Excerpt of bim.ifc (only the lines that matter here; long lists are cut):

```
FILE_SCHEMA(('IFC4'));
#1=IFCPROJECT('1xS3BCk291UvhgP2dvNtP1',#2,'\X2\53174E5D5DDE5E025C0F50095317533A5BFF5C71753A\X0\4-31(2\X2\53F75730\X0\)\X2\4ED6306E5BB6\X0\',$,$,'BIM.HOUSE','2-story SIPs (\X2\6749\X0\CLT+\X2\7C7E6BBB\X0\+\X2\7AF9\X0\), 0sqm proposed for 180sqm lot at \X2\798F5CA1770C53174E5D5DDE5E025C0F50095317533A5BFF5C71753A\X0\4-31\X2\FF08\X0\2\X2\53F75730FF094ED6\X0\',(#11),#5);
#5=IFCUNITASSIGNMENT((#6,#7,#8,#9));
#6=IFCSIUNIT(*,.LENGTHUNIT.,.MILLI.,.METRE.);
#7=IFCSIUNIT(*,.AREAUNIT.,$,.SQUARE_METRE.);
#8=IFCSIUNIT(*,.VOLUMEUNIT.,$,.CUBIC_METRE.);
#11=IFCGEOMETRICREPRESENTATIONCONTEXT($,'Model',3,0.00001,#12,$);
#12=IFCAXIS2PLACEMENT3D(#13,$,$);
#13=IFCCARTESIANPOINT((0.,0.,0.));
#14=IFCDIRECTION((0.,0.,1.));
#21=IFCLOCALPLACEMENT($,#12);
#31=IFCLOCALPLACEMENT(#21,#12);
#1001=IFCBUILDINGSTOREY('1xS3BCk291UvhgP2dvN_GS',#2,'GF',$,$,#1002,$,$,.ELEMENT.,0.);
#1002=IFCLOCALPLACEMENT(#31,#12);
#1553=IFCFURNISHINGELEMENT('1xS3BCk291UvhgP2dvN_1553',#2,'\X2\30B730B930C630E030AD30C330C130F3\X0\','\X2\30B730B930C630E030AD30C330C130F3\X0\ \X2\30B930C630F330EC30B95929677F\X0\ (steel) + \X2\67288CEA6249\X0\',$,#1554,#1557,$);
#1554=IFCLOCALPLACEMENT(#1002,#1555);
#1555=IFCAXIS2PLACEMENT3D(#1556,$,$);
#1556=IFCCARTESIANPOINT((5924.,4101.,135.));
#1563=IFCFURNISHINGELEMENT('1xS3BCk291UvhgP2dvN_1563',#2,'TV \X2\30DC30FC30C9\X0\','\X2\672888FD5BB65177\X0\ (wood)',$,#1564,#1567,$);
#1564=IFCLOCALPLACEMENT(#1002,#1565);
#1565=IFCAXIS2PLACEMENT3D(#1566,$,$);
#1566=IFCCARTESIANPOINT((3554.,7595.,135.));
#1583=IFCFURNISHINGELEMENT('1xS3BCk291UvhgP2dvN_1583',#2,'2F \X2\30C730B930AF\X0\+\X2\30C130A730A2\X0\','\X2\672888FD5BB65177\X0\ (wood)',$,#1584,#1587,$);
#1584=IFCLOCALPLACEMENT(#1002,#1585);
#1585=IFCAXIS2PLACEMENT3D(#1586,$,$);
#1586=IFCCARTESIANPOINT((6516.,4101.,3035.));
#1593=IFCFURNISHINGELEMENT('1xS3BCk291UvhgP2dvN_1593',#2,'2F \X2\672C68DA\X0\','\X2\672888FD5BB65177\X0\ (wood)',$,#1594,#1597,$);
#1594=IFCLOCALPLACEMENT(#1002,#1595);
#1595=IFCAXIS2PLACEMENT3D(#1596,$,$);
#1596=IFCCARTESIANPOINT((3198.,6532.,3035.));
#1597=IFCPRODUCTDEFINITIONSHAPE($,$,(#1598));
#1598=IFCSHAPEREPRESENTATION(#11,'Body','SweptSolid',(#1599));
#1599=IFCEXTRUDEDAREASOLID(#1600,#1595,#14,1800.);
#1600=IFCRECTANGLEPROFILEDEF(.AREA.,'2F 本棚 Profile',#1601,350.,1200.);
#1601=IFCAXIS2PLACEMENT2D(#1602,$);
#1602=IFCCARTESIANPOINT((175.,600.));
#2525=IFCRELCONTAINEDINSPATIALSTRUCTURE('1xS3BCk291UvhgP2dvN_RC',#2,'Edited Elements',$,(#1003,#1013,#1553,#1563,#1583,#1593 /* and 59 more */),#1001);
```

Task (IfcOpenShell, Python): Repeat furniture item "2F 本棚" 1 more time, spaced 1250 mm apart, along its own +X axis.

```python
import ifcopenshell
import ifcopenshell.api.geometry
import ifcopenshell.api.root
import ifcopenshell.util.element
import ifcopenshell.util.placement
import ifcopenshell.util.unit

model = ifcopenshell.open("bim.ifc")
unit_scale = ifcopenshell.util.unit.calculate_unit_scale(model)


def reuse_history(source, copy):
    """copy_class also copies each property set's owner history, people and application; keep the originals."""
    for rel in copy.IsDefinedBy:
        if rel.is_a("IfcRelDefinesByProperties") and (history := rel.RelatingPropertyDefinition.OwnerHistory):
            rel.RelatingPropertyDefinition.OwnerHistory = source.OwnerHistory
            ifcopenshell.util.element.remove_deep2(model, history)


source = model.by_guid("1xS3BCk291UvhgP2dvN_1593")
base = ifcopenshell.util.placement.get_local_placement(source.ObjectPlacement)
step = base[:3, 0] * 1.25 / unit_scale

for i in range(1, 2):
    copy = ifcopenshell.api.root.copy_class(model, product=source)
    copy.Representation = ifcopenshell.util.element.copy_deep(
        model, source.Representation, exclude=["IfcGeometricRepresentationContext", "IfcRepresentationMap"]
    )
    reuse_history(source, copy)
    matrix = base.copy()
    matrix[:3, 3] += i * step
    print("added at", matrix[:3, 3].round(3) + 0.0)
    ifcopenshell.api.geometry.edit_object_placement(model, product=copy, matrix=matrix, is_si=False)

model.write("bim-out.ifc")
```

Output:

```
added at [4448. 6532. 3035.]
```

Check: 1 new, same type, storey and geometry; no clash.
